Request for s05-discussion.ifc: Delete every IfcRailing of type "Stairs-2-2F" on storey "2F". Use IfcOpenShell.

First a look at what the model holds.

```python
import ifcopenshell
import ifcopenshell.util.element

model = ifcopenshell.open("s05-discussion.ifc")
print(model.schema)
storey = next(s for s in model.by_type("IfcBuildingStorey") if s.Name == "2F")
railings = [e for e in ifcopenshell.util.element.get_decomposition(storey) if e.is_a("IfcRailing")]
seen = {}
for e in railings:
    element_type = ifcopenshell.util.element.get_type(e)
    name = element_type.Name if element_type not in (None, e) else None
    seen[name] = seen.get(name, 0) + 1
for name, count in sorted(seen.items(), key=str):
    print(count, "x", name)
```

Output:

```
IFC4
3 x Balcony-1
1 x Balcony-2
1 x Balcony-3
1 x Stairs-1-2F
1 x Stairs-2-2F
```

```python
import ifcopenshell
import ifcopenshell.api.root
import ifcopenshell.util.element

model = ifcopenshell.open("s05-discussion.ifc")

storey = next(s for s in model.by_type("IfcBuildingStorey") if s.Name == "2F")
railings = [e for e in ifcopenshell.util.element.get_decomposition(storey) if e.is_a("IfcRailing")]
targets = [e for e in railings if (t := ifcopenshell.util.element.get_type(e)) not in (None, e) and t.Name == "Stairs-2-2F"]

for e in targets:
    ifcopenshell.api.root.remove_product(model, product=e)
print(len(targets), "removed")

model.write("s05-discussion-out.ifc")
```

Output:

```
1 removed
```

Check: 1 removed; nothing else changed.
